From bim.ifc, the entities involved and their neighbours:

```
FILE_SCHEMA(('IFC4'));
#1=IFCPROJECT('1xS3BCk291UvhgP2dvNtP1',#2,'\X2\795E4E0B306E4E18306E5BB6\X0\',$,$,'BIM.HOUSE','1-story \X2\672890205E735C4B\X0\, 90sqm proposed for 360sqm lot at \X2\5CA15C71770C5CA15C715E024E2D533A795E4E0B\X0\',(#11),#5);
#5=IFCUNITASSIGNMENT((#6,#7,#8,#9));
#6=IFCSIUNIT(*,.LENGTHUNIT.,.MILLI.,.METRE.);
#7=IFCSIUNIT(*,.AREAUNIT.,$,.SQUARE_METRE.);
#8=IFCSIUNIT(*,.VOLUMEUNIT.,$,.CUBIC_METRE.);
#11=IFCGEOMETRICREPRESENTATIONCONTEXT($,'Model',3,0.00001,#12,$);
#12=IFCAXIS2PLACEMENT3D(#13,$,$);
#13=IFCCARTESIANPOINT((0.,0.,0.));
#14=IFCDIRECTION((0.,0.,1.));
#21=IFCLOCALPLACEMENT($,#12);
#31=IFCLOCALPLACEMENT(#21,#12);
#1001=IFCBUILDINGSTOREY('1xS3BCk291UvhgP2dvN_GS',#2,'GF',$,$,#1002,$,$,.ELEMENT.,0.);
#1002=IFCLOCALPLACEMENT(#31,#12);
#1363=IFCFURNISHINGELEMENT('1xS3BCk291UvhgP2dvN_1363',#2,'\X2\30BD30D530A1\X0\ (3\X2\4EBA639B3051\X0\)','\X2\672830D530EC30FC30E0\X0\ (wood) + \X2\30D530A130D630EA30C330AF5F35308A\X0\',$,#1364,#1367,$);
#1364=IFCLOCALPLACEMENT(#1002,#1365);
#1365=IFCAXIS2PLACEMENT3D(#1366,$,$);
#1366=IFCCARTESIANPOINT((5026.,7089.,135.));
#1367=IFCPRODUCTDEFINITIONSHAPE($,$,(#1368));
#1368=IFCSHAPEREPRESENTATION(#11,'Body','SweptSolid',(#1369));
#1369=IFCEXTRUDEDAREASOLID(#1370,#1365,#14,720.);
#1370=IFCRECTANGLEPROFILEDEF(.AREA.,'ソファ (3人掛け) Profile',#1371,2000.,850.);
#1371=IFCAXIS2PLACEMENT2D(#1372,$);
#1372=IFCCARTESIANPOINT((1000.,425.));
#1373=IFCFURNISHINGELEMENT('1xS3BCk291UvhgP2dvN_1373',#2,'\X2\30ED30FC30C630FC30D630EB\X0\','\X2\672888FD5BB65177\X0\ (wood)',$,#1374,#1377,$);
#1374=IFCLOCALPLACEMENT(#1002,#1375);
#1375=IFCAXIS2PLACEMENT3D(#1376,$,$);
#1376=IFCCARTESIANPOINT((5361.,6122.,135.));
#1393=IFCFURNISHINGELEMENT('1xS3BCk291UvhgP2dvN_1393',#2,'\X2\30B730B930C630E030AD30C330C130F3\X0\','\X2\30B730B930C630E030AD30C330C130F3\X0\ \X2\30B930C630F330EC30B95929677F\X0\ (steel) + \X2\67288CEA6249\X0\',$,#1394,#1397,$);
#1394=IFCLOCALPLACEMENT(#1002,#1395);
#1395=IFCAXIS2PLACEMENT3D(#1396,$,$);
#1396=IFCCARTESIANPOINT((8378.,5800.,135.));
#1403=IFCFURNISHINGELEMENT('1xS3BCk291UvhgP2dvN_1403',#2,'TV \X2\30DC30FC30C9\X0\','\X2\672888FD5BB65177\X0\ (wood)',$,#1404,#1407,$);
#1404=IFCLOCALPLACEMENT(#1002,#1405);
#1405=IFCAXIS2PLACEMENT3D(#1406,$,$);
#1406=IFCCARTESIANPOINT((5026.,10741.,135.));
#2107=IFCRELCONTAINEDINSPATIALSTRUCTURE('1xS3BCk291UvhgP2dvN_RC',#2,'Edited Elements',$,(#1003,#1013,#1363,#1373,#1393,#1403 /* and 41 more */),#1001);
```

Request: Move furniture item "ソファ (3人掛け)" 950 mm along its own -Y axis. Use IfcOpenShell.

```python
import ifcopenshell
import ifcopenshell.api.geometry
import ifcopenshell.util.placement
import ifcopenshell.util.unit

model = ifcopenshell.open("bim.ifc")
unit_scale = ifcopenshell.util.unit.calculate_unit_scale(model)

item = model.by_guid("1xS3BCk291UvhgP2dvN_1363")
matrix = ifcopenshell.util.placement.get_local_placement(item.ObjectPlacement)
matrix[:3, 3] -= matrix[:3, 1] * 0.95 / unit_scale
ifcopenshell.api.geometry.edit_object_placement(model, product=item, matrix=matrix, is_si=False)

print(ifcopenshell.util.placement.get_local_placement(item.ObjectPlacement).round(3) + 0.0)

model.write("bim_edited.ifc")
```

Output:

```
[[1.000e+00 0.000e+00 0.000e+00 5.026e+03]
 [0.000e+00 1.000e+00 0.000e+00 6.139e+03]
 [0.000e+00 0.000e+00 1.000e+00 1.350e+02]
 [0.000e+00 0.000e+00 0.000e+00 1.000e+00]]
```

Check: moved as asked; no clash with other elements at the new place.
